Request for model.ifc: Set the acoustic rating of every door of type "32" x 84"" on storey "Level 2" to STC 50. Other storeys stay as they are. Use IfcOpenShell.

First a look at what the model holds.

```python
import ifcopenshell
import ifcopenshell.util.element

model = ifcopenshell.open("model.ifc")
print(model.schema)
storey = next(s for s in model.by_type("IfcBuildingStorey") if s.Name == "Level 2")
doors = [e for e in ifcopenshell.util.element.get_decomposition(storey) if e.is_a("IfcDoor")]
seen = {}
for e in doors:
    element_type = ifcopenshell.util.element.get_type(e)
    key = (element_type.Name if element_type != e and element_type else None, ifcopenshell.util.element.get_pset(e, "Pset_DoorCommon", "AcousticRating"))
    seen[key] = seen.get(key, 0) + 1
for (name, value), count in sorted(seen.items(), key=str):
    print(count, "x", name, "|", value)
```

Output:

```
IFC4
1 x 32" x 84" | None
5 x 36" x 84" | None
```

```python
import ifcopenshell
import ifcopenshell.api.pset
import ifcopenshell.util.element

model = ifcopenshell.open("model.ifc")

storey = next(s for s in model.by_type("IfcBuildingStorey") if s.Name == "Level 2")
doors = [e for e in ifcopenshell.util.element.get_decomposition(storey) if e.is_a("IfcDoor")]

count = 0
for e in doors:
    element_type = ifcopenshell.util.element.get_type(e)
    if element_type in (None, e) or element_type.Name != '32" x 84"':
        continue
    # add_pset returns the element's existing set when there is one.
    pset = ifcopenshell.api.pset.add_pset(model, product=e, name="Pset_DoorCommon")
    ifcopenshell.api.pset.edit_pset(model, pset=pset, properties={"AcousticRating": "STC 50"})
    count += 1

print(count, "doors updated")

model.write("model_edited.ifc")
```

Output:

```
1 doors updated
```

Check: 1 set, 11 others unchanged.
